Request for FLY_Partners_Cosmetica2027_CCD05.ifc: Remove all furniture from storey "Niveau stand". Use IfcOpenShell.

First a look at what the model holds.

```python
import ifcopenshell
import ifcopenshell.util.element

model = ifcopenshell.open("FLY_Partners_Cosmetica2027_CCD05.ifc")
print(model.schema)
storey = next(s for s in model.by_type("IfcBuildingStorey") if s.Name == "Niveau stand")
furniture = [e for e in ifcopenshell.util.element.get_decomposition(storey) if e.is_a("IfcFurnishingElement")]
seen = {}
for e in furniture:
    element_type = ifcopenshell.util.element.get_type(e)
    name = element_type.Name if element_type not in (None, e) else None
    seen[name] = seen.get(name, 0) + 1
for name, count in sorted(seen.items(), key=str):
    print(count, "x", name)
```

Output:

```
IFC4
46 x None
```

```python
import ifcopenshell
import ifcopenshell.api.root
import ifcopenshell.util.element

model = ifcopenshell.open("FLY_Partners_Cosmetica2027_CCD05.ifc")

storey = next(s for s in model.by_type("IfcBuildingStorey") if s.Name == "Niveau stand")
furniture = [e for e in ifcopenshell.util.element.get_decomposition(storey) if e.is_a("IfcFurnishingElement")]

for e in furniture:
    ifcopenshell.api.root.remove_product(model, product=e)
print(len(furniture), "removed")

model.write("FLY_Partners_Cosmetica2027_CCD05_updated.ifc")
```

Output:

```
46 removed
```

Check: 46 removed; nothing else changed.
